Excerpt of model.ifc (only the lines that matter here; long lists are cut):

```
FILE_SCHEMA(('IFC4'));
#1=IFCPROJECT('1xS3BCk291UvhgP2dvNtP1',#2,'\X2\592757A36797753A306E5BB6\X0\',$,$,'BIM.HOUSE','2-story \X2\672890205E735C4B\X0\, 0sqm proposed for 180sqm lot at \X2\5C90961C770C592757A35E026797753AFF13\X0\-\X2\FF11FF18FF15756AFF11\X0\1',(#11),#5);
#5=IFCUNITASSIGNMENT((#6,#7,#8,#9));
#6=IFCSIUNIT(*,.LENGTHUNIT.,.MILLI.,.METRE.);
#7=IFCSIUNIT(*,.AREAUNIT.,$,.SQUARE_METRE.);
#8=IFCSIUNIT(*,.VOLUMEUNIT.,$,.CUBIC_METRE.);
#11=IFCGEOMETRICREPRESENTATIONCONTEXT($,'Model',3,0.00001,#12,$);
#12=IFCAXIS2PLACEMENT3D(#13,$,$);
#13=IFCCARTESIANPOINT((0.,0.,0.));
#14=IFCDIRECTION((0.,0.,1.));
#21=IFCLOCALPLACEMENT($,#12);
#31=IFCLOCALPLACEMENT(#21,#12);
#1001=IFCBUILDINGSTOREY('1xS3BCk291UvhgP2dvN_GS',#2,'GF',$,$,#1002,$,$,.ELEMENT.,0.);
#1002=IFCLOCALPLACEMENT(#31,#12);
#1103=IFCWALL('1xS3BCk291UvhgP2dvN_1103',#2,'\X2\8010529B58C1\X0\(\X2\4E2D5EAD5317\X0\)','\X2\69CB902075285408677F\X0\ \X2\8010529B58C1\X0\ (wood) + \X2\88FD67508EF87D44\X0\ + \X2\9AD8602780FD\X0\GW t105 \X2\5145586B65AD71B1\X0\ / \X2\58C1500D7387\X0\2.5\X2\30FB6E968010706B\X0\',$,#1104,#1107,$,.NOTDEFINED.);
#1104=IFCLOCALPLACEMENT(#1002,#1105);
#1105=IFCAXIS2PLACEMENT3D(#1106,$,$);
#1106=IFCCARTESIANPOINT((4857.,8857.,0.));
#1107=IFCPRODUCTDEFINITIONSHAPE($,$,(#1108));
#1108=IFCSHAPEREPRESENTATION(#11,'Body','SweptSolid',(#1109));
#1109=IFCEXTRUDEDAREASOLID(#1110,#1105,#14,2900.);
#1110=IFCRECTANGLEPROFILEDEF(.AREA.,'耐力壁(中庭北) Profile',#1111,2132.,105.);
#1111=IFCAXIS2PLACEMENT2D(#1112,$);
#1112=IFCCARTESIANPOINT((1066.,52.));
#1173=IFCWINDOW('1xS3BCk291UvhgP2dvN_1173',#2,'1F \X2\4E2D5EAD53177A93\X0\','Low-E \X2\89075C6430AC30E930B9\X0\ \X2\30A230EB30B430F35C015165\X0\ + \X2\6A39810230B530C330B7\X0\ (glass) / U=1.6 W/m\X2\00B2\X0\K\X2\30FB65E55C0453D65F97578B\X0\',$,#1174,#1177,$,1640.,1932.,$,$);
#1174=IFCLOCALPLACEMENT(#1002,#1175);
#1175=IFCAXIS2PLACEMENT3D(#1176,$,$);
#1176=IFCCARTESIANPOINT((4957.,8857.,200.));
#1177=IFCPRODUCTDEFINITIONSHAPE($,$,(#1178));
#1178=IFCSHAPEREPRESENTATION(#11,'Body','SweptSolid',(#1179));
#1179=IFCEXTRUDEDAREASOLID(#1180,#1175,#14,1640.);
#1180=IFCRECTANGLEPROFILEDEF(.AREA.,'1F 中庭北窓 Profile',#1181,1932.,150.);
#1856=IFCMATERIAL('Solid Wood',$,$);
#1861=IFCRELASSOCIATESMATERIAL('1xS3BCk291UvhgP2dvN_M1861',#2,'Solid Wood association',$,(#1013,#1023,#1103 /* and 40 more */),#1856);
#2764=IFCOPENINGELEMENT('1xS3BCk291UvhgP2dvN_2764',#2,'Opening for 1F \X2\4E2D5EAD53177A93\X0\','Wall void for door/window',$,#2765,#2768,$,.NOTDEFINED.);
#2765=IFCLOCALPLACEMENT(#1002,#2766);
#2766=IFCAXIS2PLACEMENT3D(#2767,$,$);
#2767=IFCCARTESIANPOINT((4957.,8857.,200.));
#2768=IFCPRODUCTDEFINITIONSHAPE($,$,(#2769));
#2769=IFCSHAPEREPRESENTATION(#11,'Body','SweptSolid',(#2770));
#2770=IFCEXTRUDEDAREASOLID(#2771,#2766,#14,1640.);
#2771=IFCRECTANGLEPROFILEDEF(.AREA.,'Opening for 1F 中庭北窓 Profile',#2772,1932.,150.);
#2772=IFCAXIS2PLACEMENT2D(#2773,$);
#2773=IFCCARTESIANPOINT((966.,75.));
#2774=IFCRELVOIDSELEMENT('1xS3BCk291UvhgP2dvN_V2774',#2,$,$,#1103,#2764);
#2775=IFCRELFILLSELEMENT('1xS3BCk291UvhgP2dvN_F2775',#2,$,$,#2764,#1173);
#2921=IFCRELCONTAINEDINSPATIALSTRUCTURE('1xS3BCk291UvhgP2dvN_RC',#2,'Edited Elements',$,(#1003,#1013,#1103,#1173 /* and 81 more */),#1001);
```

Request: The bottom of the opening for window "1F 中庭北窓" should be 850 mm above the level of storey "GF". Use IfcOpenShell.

```python
import numpy as np
import ifcopenshell
import ifcopenshell.api.geometry
import ifcopenshell.geom
import ifcopenshell.util.element
import ifcopenshell.util.placement
import ifcopenshell.util.shape
import ifcopenshell.util.unit

model = ifcopenshell.open("model.ifc")
unit_scale = ifcopenshell.util.unit.calculate_unit_scale(model)

window = model.by_guid("1xS3BCk291UvhgP2dvN_1173")
opening = window.FillsVoids[0].RelatingOpeningElement
storey = ifcopenshell.util.element.get_container(window, ifc_class="IfcBuildingStorey")
level = ifcopenshell.util.placement.get_local_placement(storey.ObjectPlacement)[2, 3]

# The opening's origin need not be at the sill, so measure its lowest point.
shape = ifcopenshell.geom.create_shape(ifcopenshell.geom.settings(), opening)
bottom = ifcopenshell.util.shape.get_shape_bottom_elevation(shape, shape.geometry) / unit_scale
dz = level + 850.0 - bottom

shift = np.array([0.0, 0.0, dz])
# The window is not placed relative to its opening, so move both.
for product in (opening, window):
    matrix = ifcopenshell.util.placement.get_local_placement(product.ObjectPlacement)
    matrix[:3, 3] += shift
    ifcopenshell.api.geometry.edit_object_placement(model, product=product, matrix=matrix, is_si=False)

print(f"moved by {dz * unit_scale:+.3f} m")

model.write("model_v2.ifc")
```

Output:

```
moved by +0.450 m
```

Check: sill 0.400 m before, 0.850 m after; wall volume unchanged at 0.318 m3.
